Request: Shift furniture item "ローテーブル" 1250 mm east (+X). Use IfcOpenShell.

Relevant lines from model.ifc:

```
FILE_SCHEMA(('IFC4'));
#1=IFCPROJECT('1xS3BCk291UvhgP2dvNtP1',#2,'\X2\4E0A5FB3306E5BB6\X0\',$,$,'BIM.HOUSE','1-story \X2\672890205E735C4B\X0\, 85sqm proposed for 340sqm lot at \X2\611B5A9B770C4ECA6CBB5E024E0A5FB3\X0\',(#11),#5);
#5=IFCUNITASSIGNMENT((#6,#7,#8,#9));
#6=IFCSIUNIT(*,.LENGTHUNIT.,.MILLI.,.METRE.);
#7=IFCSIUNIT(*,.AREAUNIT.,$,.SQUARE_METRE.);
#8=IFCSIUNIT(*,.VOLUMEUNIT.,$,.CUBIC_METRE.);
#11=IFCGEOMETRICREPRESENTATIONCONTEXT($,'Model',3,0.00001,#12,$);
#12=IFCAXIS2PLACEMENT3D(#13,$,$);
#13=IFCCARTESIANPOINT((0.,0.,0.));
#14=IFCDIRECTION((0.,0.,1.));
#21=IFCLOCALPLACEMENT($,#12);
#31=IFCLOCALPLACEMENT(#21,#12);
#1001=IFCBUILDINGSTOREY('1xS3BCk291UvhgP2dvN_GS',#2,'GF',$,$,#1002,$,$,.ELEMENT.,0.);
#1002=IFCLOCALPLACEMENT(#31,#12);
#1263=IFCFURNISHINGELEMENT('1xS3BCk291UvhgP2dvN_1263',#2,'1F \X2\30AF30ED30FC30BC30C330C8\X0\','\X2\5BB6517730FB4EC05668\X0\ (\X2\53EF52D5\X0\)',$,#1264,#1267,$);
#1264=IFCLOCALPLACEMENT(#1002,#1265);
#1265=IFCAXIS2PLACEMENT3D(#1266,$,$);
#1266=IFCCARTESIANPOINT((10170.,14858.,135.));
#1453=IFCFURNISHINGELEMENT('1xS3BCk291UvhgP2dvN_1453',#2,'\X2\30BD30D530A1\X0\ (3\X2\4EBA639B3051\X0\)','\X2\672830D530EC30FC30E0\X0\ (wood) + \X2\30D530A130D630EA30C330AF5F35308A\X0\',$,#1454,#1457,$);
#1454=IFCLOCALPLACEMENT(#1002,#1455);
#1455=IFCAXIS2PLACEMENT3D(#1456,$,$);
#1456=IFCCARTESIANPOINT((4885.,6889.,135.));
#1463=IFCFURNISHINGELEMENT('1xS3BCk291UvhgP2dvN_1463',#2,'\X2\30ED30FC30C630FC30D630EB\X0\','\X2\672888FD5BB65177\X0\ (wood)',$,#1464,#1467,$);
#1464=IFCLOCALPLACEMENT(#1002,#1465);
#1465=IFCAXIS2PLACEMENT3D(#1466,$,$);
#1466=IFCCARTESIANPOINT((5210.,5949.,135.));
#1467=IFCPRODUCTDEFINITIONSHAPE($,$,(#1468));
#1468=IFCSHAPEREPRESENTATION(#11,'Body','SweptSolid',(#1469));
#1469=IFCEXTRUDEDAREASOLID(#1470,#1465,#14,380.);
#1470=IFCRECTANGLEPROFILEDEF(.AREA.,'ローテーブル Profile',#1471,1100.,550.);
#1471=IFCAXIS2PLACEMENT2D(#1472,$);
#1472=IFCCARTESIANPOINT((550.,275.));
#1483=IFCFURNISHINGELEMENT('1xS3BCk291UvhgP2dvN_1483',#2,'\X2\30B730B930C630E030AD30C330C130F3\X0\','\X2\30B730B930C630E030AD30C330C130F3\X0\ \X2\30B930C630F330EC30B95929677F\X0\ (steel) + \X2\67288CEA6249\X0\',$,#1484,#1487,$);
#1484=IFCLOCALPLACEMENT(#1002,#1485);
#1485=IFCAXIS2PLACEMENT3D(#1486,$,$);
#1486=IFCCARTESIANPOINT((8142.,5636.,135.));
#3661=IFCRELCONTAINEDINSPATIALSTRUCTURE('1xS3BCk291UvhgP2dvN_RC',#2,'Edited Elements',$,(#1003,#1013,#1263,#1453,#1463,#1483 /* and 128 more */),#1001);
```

```python
import ifcopenshell
import ifcopenshell.api.geometry
import ifcopenshell.util.placement
import ifcopenshell.util.unit

model = ifcopenshell.open("model.ifc")
unit_scale = ifcopenshell.util.unit.calculate_unit_scale(model)

item = model.by_guid("1xS3BCk291UvhgP2dvN_1463")
matrix = ifcopenshell.util.placement.get_local_placement(item.ObjectPlacement)
matrix[0, 3] += 1.25 / unit_scale
ifcopenshell.api.geometry.edit_object_placement(model, product=item, matrix=matrix, is_si=False)

print(ifcopenshell.util.placement.get_local_placement(item.ObjectPlacement).round(3) + 0.0)

model.write("model_rev.ifc")
```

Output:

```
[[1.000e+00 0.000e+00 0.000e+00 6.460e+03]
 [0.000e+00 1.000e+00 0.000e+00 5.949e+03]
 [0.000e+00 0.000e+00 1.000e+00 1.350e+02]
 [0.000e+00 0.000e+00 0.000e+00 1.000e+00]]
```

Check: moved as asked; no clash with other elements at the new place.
